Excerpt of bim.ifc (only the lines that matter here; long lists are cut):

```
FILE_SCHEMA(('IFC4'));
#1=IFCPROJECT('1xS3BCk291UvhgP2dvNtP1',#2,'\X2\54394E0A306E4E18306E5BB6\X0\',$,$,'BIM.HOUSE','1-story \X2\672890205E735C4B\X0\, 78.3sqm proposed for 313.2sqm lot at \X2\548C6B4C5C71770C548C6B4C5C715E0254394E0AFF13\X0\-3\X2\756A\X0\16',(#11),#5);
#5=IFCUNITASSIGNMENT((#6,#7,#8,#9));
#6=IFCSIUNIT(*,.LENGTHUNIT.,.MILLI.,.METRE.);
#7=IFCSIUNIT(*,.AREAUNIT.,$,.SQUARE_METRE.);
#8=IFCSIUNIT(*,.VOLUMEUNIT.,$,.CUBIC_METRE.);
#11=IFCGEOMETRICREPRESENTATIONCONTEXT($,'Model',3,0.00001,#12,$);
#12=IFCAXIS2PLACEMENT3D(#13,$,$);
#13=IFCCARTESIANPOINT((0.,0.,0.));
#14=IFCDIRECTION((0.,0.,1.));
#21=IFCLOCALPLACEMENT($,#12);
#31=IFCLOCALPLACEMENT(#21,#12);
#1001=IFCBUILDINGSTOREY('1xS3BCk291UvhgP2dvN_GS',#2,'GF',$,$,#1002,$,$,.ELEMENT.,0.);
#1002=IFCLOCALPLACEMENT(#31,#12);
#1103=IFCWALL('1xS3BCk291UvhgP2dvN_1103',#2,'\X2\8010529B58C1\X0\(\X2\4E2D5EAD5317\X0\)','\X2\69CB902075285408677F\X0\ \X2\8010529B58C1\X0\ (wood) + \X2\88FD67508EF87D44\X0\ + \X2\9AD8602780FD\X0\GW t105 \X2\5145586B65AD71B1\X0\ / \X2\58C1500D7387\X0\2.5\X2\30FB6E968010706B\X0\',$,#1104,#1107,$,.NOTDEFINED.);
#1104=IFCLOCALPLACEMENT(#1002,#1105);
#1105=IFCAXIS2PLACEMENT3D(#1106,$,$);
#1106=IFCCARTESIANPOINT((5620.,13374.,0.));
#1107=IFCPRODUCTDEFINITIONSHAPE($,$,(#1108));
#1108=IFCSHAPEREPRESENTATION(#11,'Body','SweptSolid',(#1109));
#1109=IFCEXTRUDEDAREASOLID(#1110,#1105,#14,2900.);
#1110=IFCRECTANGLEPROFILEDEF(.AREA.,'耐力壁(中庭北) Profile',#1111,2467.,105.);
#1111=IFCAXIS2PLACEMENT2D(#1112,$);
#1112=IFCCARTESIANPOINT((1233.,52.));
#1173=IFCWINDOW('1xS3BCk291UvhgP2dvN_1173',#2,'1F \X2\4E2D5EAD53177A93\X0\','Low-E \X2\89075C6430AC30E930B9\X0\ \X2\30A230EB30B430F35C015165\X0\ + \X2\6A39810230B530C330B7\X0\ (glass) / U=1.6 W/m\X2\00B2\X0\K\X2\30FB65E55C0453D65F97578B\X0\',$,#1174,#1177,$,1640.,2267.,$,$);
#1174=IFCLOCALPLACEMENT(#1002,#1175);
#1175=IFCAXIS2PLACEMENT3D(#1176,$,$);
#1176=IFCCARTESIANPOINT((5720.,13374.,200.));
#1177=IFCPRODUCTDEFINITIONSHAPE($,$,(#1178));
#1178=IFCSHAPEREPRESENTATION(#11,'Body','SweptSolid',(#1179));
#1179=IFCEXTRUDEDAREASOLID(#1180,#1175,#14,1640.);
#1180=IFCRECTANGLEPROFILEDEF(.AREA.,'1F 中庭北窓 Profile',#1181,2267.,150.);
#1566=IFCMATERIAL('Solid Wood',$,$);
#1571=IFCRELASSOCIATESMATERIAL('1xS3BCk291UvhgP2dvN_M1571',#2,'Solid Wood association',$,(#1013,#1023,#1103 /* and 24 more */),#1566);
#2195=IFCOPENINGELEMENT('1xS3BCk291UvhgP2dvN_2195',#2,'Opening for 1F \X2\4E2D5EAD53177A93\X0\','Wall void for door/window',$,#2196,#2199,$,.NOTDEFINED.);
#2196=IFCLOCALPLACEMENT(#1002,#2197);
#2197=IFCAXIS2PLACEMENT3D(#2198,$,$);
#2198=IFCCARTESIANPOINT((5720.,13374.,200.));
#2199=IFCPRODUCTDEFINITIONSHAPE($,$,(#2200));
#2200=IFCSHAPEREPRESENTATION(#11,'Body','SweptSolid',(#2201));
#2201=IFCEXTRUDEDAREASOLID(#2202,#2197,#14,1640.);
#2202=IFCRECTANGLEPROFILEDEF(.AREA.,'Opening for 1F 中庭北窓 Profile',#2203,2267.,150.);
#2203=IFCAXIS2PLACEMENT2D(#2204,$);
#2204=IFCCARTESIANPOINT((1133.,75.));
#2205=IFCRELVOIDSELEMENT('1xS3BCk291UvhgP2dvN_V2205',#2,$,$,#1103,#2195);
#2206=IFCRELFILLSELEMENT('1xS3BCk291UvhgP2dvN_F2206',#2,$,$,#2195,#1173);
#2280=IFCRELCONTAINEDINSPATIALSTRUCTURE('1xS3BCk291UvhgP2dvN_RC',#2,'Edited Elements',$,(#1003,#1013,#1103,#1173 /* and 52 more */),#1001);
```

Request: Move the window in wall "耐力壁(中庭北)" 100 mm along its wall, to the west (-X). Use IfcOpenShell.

```python
import ifcopenshell
import ifcopenshell.api.geometry
import ifcopenshell.util.placement

model = ifcopenshell.open("bim.ifc")

window = model.by_guid("1xS3BCk291UvhgP2dvN_1173")
opening = window.FillsVoids[0].RelatingOpeningElement
wall = opening.VoidsElements[0].RelatingBuildingElement

wall_matrix = ifcopenshell.util.placement.get_local_placement(wall.ObjectPlacement)
shift = wall_matrix[:3, 0] * -100.0
before = ifcopenshell.util.placement.get_local_placement(window.ObjectPlacement)[:3, 3].copy()

# The window is not placed relative to its opening, so move both.
for product in (opening, window):
    matrix = ifcopenshell.util.placement.get_local_placement(product.ObjectPlacement)
    matrix[:3, 3] += shift
    ifcopenshell.api.geometry.edit_object_placement(model, product=product, matrix=matrix, is_si=False)

after = ifcopenshell.util.placement.get_local_placement(window.ObjectPlacement)[:3, 3]
print("window moved by", (after - before).round(3) + 0.0)

model.write("bim_rev.ifc")
```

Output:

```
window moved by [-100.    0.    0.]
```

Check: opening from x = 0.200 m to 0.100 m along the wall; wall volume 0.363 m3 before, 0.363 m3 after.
